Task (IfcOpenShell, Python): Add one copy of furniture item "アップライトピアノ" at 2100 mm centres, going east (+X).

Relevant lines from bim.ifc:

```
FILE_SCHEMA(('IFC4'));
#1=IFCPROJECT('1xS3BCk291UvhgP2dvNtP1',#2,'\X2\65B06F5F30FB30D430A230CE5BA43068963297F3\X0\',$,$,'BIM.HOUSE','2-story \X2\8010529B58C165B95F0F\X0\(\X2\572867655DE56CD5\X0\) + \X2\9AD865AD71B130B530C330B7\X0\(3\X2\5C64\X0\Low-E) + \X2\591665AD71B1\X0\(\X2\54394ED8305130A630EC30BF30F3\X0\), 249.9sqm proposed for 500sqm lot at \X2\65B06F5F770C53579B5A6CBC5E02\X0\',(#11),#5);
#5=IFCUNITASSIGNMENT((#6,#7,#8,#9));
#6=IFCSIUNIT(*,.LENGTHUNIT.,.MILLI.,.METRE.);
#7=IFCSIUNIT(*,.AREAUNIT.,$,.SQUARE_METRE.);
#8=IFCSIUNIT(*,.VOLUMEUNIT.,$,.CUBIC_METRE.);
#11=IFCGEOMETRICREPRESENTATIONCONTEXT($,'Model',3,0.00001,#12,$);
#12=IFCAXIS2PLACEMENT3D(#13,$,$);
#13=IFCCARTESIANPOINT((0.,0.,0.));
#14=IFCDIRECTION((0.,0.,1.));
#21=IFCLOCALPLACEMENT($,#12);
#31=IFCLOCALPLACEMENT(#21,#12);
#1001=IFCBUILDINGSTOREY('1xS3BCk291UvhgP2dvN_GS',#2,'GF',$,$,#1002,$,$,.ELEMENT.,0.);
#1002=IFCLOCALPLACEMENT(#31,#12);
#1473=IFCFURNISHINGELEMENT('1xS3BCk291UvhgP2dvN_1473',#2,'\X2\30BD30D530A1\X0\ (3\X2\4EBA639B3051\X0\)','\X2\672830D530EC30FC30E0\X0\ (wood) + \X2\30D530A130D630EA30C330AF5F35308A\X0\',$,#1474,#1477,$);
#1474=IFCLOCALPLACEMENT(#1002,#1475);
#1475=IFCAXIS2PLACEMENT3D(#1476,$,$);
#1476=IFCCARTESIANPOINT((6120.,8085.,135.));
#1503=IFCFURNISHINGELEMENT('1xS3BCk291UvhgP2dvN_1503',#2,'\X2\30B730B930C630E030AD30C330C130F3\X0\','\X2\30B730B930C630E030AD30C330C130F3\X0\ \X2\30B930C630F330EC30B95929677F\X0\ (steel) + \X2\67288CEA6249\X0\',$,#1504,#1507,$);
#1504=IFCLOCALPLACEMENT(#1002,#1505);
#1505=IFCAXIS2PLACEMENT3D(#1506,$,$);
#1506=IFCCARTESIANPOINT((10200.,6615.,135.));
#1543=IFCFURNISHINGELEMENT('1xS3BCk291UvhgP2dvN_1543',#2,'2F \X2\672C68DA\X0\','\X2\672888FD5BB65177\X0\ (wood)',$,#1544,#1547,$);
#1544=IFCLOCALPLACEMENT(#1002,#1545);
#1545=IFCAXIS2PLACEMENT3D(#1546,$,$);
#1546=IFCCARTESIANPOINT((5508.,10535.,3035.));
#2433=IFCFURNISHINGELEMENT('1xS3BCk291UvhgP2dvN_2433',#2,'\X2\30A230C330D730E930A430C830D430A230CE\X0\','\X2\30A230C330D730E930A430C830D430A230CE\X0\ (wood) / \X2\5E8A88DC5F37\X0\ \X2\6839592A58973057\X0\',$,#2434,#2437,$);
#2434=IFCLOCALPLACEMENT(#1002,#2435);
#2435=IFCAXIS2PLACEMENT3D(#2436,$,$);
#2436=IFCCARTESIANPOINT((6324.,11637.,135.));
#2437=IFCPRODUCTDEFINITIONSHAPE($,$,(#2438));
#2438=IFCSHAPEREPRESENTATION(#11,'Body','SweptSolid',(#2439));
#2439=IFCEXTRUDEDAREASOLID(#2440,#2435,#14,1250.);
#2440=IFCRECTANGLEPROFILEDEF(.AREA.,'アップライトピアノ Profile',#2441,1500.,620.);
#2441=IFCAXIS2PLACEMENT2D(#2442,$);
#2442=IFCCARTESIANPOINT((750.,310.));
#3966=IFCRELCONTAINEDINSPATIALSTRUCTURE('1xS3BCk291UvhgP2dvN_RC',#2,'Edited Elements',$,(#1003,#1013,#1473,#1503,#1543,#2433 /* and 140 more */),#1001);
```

```python
import numpy as np
import ifcopenshell
import ifcopenshell.api.geometry
import ifcopenshell.api.root
import ifcopenshell.util.element
import ifcopenshell.util.placement
import ifcopenshell.util.unit

model = ifcopenshell.open("bim.ifc")
unit_scale = ifcopenshell.util.unit.calculate_unit_scale(model)


def reuse_history(source, copy):
    """copy_class also copies each property set's owner history, people and application; keep the originals."""
    for rel in copy.IsDefinedBy:
        if rel.is_a("IfcRelDefinesByProperties") and (history := rel.RelatingPropertyDefinition.OwnerHistory):
            rel.RelatingPropertyDefinition.OwnerHistory = source.OwnerHistory
            ifcopenshell.util.element.remove_deep2(model, history)


source = model.by_id(2433)
base = ifcopenshell.util.placement.get_local_placement(source.ObjectPlacement)
step = np.array([1.0, 0.0, 0.0]) * 2.1 / unit_scale

for i in range(1, 2):
    copy = ifcopenshell.api.root.copy_class(model, product=source)
    copy.Representation = ifcopenshell.util.element.copy_deep(
        model, source.Representation, exclude=["IfcGeometricRepresentationContext", "IfcRepresentationMap"]
    )
    reuse_history(source, copy)
    matrix = base.copy()
    matrix[:3, 3] += i * step
    print("added at", matrix[:3, 3].round(3) + 0.0)
    ifcopenshell.api.geometry.edit_object_placement(model, product=copy, matrix=matrix, is_si=False)

model.write("bim_rev.ifc")
```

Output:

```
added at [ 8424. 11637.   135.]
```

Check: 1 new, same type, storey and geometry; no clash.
